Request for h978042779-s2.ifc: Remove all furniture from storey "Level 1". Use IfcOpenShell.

First a look at what the model holds.

```python
import ifcopenshell
import ifcopenshell.util.element

model = ifcopenshell.open("h978042779-s2.ifc")
print(model.schema)
storey = next(s for s in model.by_type("IfcBuildingStorey") if s.Name == "Level 1")
furniture = [e for e in ifcopenshell.util.element.get_decomposition(storey) if e.is_a("IfcFurnishingElement")]
seen = {}
for e in furniture:
    element_type = ifcopenshell.util.element.get_type(e)
    name = element_type.Name if element_type not in (None, e) else None
    seen[name] = seen.get(name, 0) + 1
for name, count in sorted(seen.items(), key=str):
    print(count, "x", name)
```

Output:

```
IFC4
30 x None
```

```python
import ifcopenshell
import ifcopenshell.api.root
import ifcopenshell.util.element

model = ifcopenshell.open("h978042779-s2.ifc")

storey = next(s for s in model.by_type("IfcBuildingStorey") if s.Name == "Level 1")
furniture = [e for e in ifcopenshell.util.element.get_decomposition(storey) if e.is_a("IfcFurnishingElement")]

for e in furniture:
    ifcopenshell.api.root.remove_product(model, product=e)
print(len(furniture), "removed")

model.write("h978042779-s2_edited.ifc")
```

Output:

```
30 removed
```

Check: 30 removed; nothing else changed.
